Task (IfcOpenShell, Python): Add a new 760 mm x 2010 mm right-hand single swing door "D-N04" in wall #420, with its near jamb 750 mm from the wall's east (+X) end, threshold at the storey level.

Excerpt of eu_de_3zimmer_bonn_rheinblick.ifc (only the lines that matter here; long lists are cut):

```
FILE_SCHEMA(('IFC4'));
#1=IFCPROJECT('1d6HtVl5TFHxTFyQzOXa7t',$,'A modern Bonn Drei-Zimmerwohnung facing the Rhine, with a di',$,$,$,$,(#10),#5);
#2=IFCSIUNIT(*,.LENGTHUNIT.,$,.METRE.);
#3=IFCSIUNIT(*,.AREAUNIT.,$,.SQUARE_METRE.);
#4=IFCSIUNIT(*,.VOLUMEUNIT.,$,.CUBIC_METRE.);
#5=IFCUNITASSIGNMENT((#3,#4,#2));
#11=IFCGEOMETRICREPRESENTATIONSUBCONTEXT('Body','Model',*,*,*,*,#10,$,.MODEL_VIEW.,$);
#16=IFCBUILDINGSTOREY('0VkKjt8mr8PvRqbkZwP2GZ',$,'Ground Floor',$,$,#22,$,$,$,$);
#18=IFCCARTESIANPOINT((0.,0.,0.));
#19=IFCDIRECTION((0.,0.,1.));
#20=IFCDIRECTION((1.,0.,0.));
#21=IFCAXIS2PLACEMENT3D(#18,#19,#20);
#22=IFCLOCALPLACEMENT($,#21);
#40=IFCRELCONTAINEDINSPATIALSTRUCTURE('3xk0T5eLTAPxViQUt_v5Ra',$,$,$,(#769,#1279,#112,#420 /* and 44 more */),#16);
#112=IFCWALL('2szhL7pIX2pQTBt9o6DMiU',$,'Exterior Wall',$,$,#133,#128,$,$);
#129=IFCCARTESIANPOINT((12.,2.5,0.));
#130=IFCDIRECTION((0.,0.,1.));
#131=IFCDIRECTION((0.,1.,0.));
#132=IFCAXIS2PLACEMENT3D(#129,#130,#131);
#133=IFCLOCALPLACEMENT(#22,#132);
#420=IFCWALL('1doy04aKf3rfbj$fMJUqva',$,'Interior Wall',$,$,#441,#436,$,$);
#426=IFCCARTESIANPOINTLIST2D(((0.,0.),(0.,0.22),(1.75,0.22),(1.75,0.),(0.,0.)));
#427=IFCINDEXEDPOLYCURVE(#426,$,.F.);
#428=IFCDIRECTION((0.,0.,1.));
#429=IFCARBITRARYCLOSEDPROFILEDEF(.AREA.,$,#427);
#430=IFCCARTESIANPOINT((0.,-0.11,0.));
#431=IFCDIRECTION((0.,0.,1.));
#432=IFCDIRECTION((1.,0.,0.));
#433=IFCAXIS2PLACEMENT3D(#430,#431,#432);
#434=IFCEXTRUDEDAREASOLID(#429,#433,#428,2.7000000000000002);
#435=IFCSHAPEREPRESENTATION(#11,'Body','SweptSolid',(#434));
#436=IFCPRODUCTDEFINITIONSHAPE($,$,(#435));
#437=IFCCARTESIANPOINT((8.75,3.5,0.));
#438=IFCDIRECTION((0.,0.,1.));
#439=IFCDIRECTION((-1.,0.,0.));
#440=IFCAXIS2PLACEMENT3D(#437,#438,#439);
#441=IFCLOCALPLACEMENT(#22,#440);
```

```python
import numpy as np
import ifcopenshell
import ifcopenshell.api.feature
import ifcopenshell.api.geometry
import ifcopenshell.api.root
import ifcopenshell.api.spatial
import ifcopenshell.geom
import ifcopenshell.util.element
import ifcopenshell.util.placement
import ifcopenshell.util.representation
import ifcopenshell.util.shape
import ifcopenshell.util.unit

model = ifcopenshell.open("eu_de_3zimmer_bonn_rheinblick.ifc")
unit_scale = ifcopenshell.util.unit.calculate_unit_scale(model)
settings = ifcopenshell.geom.settings()


def volume(element):
    """Net volume in cubic metres, openings subtracted."""
    shape = ifcopenshell.geom.create_shape(settings, element)
    return ifcopenshell.util.shape.get_volume(shape.geometry)


wall = model.by_guid("1doy04aKf3rfbj$fMJUqva")
storey = ifcopenshell.util.element.get_container(wall, ifc_class="IfcBuildingStorey")
context = ifcopenshell.util.representation.get_context(model, "Model", "Body", "MODEL_VIEW")
before = volume(wall)

width, height, from_end, sill = 0.76, 2.01, 0.75, 0.0  # metres

# The wall runs along its own X axis, and the end named is its -X end.
wall_shape = ifcopenshell.geom.create_shape(settings, wall)
x, y, z = ifcopenshell.util.shape.get_vertices(wall_shape.geometry).T
start = x.min() + from_end
face, thickness = float(y.min()), float(y.max() - y.min())
wall_matrix = ifcopenshell.util.placement.get_local_placement(wall.ObjectPlacement)
level = ifcopenshell.util.placement.get_local_placement(storey.ObjectPlacement)[2, 3]


def in_wall(x, y):
    """Placement at x, y metres in the wall's axes, at sill height."""
    matrix = wall_matrix.copy()
    matrix[:, 3] = wall_matrix @ np.array([x / unit_scale, y / unit_scale, 0.0, 1.0])
    matrix[2, 3] = level + sill / unit_scale
    return matrix


# Opening: a box that overshoots both wall faces by 50 mm.
opening = ifcopenshell.api.root.create_entity(model, ifc_class="IfcOpeningElement", predefined_type="OPENING")
box = ifcopenshell.api.geometry.add_wall_representation(
    model, context=context, length=width, height=height, thickness=thickness + 0.1
)
ifcopenshell.api.geometry.assign_representation(model, product=opening, representation=box)
ifcopenshell.api.geometry.edit_object_placement(model, product=opening, matrix=in_wall(start, face - 0.05), is_si=False)
ifcopenshell.api.feature.add_feature(model, feature=opening, element=wall)

door = ifcopenshell.api.root.create_entity(model, ifc_class="IfcDoor", name="D-N04", predefined_type="DOOR")
door.OverallWidth, door.OverallHeight = width / unit_scale, height / unit_scale
door.OperationType = "SINGLE_SWING_RIGHT"
body = ifcopenshell.api.geometry.add_door_representation(
    model,
    context=context,
    overall_width=door.OverallWidth,
    overall_height=door.OverallHeight,
    operation_type="SINGLE_SWING_RIGHT",
    lining_properties={"LiningDepth": thickness / unit_scale, "ThresholdDepth": thickness / unit_scale},
)
ifcopenshell.api.geometry.assign_representation(model, product=door, representation=body)
ifcopenshell.api.spatial.assign_container(model, products=[door], relating_structure=storey)
ifcopenshell.api.feature.add_filling(model, opening=opening, element=door)

# The lining spans the wall, so the door starts at the wall face.
ifcopenshell.api.geometry.edit_object_placement(model, product=door, matrix=in_wall(start, face), is_si=False)

after = volume(wall)

print(f"wall volume {before:.3f} -> {after:.3f} m3")

model.write("eu_de_3zimmer_bonn_rheinblick_edited.ifc")
```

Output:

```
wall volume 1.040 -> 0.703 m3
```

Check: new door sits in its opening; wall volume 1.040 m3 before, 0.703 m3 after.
